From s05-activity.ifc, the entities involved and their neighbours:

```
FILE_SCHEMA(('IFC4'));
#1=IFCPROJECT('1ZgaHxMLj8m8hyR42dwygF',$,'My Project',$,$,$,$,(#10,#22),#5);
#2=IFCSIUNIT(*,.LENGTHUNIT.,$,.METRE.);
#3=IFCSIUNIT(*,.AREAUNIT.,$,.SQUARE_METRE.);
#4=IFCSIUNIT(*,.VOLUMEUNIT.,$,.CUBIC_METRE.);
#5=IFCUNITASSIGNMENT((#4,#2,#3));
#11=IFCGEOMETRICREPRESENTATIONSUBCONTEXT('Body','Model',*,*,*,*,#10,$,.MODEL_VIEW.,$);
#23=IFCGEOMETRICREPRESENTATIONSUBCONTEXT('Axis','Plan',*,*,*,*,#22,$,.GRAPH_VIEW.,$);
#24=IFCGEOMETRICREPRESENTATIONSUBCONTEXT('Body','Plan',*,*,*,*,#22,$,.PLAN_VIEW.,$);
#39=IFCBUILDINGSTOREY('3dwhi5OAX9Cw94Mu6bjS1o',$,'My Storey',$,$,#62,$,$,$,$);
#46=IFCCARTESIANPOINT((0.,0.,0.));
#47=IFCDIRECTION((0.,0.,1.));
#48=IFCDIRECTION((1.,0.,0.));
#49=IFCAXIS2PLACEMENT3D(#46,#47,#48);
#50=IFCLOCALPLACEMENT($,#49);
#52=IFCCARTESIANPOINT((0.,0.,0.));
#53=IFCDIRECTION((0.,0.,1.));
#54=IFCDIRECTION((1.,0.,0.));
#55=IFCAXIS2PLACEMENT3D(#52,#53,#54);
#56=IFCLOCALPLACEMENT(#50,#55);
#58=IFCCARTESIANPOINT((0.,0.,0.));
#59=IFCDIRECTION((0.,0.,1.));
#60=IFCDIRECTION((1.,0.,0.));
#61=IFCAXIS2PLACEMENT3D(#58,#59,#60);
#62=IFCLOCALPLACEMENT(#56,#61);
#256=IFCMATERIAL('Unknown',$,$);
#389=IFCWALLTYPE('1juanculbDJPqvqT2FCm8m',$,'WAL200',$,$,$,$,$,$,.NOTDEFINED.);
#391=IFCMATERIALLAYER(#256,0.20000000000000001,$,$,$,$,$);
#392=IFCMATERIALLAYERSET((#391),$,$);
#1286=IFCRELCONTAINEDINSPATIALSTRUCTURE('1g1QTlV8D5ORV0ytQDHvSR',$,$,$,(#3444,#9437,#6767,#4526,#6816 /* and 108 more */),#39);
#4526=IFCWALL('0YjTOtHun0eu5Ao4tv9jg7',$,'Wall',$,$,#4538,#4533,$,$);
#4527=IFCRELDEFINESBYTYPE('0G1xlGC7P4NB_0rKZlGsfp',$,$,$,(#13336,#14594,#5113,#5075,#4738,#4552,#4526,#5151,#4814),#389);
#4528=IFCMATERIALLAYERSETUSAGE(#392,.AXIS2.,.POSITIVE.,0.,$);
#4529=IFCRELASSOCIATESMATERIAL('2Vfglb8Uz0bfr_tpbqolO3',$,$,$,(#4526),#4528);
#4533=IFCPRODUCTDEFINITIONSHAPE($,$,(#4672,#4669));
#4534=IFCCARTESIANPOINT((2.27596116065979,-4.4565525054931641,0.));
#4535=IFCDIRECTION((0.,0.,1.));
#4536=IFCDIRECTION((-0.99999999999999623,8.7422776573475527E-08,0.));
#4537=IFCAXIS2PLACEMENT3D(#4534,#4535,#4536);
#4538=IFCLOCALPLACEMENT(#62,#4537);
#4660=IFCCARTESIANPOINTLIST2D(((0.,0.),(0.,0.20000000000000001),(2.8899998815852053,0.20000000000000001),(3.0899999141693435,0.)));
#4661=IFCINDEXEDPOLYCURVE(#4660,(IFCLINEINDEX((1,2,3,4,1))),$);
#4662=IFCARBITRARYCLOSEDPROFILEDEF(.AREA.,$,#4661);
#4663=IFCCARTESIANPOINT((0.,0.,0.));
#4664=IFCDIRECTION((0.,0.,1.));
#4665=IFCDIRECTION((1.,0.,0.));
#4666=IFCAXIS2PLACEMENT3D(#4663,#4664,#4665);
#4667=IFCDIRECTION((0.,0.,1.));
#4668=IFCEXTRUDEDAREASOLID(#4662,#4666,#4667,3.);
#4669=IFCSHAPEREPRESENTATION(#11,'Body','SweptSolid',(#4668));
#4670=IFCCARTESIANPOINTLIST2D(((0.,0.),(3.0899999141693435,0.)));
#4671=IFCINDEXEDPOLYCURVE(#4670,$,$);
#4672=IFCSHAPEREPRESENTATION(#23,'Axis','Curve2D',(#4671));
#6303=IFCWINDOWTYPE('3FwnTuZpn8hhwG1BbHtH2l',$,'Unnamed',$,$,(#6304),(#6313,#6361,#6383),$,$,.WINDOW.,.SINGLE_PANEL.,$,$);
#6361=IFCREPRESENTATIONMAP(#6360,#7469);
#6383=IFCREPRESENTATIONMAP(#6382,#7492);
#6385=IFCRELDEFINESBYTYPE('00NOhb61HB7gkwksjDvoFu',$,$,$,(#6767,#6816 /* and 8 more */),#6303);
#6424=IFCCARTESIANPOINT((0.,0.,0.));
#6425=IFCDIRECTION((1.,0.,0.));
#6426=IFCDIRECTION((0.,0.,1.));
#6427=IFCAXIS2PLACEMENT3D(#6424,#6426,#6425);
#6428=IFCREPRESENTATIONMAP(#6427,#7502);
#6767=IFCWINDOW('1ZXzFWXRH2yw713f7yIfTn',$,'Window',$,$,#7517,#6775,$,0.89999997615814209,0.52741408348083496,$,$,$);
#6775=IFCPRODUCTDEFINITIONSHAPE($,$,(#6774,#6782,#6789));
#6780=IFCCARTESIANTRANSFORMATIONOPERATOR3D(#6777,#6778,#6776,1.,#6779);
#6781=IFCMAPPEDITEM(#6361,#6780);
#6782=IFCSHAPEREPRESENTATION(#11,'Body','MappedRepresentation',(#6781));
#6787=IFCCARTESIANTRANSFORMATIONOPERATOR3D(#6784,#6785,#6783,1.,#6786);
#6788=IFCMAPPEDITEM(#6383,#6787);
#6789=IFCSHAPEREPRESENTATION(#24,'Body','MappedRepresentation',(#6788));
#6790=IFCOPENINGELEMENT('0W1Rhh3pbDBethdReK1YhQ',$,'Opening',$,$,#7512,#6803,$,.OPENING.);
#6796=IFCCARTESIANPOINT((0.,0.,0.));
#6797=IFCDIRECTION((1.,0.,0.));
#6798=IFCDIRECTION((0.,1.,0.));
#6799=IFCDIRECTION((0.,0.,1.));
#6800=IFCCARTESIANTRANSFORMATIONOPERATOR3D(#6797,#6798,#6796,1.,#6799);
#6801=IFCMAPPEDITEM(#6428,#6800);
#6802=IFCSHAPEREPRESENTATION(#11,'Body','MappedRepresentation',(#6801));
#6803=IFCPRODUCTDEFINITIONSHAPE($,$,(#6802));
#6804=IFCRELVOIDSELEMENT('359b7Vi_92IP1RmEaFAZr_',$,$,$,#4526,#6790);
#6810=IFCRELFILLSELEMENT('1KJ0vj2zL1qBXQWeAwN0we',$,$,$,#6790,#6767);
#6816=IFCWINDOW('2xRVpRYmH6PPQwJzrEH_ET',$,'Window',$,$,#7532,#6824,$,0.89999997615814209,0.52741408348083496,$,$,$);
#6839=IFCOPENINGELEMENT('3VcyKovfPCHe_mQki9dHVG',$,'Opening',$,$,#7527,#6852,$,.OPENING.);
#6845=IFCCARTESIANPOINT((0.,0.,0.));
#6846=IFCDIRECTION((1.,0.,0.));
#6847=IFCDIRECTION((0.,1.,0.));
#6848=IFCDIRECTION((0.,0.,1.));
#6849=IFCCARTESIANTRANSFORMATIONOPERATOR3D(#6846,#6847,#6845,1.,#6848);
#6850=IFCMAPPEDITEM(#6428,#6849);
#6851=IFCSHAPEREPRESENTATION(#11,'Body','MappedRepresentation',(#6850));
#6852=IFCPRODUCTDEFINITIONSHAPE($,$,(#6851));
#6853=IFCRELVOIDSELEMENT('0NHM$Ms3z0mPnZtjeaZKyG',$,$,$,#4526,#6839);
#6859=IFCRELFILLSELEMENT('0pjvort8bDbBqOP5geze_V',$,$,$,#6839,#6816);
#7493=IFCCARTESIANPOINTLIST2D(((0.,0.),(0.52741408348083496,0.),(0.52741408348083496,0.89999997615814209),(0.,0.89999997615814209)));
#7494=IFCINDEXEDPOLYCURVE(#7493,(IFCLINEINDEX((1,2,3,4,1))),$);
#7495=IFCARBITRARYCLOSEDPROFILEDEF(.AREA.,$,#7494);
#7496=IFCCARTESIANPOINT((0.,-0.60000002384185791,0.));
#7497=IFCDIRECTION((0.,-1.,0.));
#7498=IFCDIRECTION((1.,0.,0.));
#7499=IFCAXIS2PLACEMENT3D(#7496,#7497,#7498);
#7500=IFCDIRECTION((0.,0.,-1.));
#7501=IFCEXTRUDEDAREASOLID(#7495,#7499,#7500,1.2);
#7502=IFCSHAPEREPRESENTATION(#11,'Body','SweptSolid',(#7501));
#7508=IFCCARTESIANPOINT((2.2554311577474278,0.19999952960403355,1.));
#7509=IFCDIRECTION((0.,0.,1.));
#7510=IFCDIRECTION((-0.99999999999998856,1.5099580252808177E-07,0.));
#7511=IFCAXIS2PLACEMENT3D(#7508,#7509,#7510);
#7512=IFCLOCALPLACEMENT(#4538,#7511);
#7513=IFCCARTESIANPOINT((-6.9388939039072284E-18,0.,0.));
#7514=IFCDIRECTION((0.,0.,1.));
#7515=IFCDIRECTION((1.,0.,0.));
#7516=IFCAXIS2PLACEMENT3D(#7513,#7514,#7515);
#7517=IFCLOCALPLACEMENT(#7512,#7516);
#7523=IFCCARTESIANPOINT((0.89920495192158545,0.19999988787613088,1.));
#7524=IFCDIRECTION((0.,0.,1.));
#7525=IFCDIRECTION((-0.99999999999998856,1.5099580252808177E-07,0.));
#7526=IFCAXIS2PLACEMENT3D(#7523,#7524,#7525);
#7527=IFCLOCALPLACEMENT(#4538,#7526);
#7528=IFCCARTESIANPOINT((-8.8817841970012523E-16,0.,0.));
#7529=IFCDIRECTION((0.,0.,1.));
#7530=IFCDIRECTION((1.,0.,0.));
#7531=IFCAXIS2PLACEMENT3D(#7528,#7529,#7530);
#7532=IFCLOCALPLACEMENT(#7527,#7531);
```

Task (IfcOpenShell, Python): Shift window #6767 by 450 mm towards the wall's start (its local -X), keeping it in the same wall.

```python
import ifcopenshell
import ifcopenshell.api.geometry
import ifcopenshell.util.placement
import ifcopenshell.util.unit

model = ifcopenshell.open("s05-activity.ifc")
unit_scale = ifcopenshell.util.unit.calculate_unit_scale(model)

window = model.by_guid("1ZXzFWXRH2yw713f7yIfTn")
opening = window.FillsVoids[0].RelatingOpeningElement
wall = opening.VoidsElements[0].RelatingBuildingElement

wall_matrix = ifcopenshell.util.placement.get_local_placement(wall.ObjectPlacement)
shift = wall_matrix[:3, 0] * -0.45 / unit_scale
before = ifcopenshell.util.placement.get_local_placement(window.ObjectPlacement)[:3, 3].copy()

# The window is placed relative to its opening, so it follows when the opening moves.
matrix = ifcopenshell.util.placement.get_local_placement(opening.ObjectPlacement)
matrix[:3, 3] += shift
ifcopenshell.api.geometry.edit_object_placement(
    model, product=opening, matrix=matrix, is_si=False, should_transform_children=True
)

after = ifcopenshell.util.placement.get_local_placement(window.ObjectPlacement)[:3, 3]
print("window moved by", (after - before).round(3) + 0.0)

model.write("s05-activity-out.ifc")
```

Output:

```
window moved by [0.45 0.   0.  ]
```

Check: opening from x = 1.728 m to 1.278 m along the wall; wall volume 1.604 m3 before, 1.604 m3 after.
